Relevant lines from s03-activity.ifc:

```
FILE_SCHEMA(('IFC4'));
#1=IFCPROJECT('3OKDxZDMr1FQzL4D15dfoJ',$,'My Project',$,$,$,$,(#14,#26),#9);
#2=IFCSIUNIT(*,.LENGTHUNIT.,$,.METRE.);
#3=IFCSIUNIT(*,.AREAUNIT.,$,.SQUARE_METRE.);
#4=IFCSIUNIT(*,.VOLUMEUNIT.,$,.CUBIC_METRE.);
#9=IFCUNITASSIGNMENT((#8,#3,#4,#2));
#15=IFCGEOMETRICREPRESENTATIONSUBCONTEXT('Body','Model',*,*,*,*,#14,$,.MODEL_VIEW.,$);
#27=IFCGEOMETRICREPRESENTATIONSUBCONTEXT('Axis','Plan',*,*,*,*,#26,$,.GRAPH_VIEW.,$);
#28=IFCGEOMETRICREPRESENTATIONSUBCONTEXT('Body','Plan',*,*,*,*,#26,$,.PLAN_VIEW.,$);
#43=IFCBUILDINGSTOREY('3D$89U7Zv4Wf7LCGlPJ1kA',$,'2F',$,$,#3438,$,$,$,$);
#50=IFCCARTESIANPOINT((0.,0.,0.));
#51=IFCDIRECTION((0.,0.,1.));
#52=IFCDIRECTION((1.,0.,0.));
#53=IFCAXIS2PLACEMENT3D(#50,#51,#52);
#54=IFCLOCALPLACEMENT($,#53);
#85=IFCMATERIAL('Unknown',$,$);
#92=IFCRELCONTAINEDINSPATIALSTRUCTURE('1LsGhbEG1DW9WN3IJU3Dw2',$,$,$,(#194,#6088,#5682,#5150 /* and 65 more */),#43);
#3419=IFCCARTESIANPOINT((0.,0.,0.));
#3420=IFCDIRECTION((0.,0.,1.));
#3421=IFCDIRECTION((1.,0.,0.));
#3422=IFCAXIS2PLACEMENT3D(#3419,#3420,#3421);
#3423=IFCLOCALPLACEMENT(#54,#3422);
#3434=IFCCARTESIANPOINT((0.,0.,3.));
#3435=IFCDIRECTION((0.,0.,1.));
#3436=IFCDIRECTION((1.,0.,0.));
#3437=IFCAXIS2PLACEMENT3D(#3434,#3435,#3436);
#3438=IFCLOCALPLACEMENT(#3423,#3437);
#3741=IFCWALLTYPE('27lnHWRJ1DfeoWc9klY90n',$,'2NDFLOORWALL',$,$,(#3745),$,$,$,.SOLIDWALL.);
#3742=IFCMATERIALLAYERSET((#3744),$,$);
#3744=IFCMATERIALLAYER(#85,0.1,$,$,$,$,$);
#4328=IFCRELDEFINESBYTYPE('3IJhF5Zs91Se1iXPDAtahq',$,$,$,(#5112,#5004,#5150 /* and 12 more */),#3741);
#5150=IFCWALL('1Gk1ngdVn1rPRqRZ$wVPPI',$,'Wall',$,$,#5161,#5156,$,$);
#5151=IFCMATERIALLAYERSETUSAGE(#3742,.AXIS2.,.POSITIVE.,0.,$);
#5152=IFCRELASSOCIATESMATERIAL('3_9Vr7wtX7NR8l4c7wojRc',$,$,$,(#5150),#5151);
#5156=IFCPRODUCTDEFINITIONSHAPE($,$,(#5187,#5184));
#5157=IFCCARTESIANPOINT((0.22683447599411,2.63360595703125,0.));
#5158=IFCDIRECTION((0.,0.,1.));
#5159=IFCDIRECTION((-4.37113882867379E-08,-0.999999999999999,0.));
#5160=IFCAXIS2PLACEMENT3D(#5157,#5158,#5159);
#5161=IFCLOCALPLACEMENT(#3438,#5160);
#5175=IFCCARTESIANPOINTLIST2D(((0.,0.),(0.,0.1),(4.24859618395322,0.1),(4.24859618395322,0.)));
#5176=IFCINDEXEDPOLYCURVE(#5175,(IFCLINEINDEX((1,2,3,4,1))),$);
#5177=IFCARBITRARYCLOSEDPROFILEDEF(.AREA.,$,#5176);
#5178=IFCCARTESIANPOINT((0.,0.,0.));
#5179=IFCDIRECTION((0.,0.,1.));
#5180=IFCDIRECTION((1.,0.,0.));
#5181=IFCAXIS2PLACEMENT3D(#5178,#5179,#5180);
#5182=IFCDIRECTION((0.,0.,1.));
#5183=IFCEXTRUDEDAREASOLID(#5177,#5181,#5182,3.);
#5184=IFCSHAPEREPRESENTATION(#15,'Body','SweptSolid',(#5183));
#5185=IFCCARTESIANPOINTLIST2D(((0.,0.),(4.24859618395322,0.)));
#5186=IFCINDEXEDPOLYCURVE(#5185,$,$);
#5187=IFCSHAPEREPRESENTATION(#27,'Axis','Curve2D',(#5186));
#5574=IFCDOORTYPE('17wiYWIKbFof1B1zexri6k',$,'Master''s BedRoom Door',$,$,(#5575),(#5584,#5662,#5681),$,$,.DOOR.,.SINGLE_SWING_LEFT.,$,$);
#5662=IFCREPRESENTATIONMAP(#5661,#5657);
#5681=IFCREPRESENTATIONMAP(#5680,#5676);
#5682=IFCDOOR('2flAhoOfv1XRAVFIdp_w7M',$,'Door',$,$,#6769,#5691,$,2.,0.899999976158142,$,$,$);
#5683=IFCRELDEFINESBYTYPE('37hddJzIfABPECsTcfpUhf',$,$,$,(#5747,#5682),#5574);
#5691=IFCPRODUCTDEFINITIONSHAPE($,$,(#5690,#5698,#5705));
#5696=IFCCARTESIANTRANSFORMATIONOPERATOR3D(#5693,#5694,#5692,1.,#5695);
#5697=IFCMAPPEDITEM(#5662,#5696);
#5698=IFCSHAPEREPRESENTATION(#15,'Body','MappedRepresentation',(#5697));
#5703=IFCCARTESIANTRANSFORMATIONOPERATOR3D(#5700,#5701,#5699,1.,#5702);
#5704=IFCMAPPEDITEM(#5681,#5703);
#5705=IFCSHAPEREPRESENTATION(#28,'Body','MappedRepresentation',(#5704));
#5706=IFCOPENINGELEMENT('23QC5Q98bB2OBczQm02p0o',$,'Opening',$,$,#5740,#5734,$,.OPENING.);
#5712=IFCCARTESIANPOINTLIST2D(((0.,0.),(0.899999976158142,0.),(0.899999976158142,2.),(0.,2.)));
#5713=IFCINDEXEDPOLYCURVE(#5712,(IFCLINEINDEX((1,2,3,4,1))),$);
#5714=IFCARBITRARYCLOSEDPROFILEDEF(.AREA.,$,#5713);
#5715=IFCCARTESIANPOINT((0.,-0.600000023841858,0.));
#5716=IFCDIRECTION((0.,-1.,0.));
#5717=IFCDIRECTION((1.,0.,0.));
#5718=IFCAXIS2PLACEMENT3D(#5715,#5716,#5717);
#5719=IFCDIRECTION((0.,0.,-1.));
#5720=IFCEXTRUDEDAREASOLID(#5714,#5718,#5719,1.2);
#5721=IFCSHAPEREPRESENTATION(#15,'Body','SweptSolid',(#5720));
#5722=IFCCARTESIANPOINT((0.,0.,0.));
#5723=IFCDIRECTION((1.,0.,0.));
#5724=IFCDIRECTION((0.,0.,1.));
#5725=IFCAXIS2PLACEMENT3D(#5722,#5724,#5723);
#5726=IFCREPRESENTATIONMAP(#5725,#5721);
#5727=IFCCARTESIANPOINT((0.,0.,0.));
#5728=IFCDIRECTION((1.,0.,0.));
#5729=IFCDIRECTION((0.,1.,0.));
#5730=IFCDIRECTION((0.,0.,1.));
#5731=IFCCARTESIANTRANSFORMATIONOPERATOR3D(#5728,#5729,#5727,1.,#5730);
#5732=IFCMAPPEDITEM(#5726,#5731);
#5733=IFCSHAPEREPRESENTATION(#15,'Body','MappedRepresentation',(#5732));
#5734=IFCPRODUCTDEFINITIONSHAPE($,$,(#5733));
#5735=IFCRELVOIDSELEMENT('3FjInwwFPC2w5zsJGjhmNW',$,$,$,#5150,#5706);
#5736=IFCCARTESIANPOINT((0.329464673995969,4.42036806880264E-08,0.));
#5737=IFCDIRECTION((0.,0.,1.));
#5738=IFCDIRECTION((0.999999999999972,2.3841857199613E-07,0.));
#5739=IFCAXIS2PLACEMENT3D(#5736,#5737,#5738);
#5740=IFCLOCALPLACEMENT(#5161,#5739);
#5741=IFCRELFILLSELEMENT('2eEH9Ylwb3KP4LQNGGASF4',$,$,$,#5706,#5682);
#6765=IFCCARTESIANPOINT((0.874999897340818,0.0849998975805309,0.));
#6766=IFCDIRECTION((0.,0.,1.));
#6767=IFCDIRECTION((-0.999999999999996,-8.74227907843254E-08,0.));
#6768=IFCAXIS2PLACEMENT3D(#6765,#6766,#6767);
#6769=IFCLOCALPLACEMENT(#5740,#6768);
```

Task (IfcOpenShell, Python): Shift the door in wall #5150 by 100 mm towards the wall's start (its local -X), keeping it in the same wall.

```python
import ifcopenshell
import ifcopenshell.api.geometry
import ifcopenshell.util.placement

model = ifcopenshell.open("s03-activity.ifc")

door = model.by_guid("2flAhoOfv1XRAVFIdp_w7M")
opening = door.FillsVoids[0].RelatingOpeningElement
wall = opening.VoidsElements[0].RelatingBuildingElement

wall_matrix = ifcopenshell.util.placement.get_local_placement(wall.ObjectPlacement)
shift = wall_matrix[:3, 0] * -0.1
before = ifcopenshell.util.placement.get_local_placement(door.ObjectPlacement)[:3, 3].copy()

# The door is placed relative to its opening, so it follows when the opening moves.
matrix = ifcopenshell.util.placement.get_local_placement(opening.ObjectPlacement)
matrix[:3, 3] += shift
ifcopenshell.api.geometry.edit_object_placement(
    model, product=opening, matrix=matrix, is_si=False, should_transform_children=True
)

after = ifcopenshell.util.placement.get_local_placement(door.ObjectPlacement)[:3, 3]
print("door moved by", (after - before).round(3) + 0.0)

model.write("s03-activity_rev.ifc")
```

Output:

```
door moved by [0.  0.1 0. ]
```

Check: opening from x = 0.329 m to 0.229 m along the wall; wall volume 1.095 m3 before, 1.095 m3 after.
